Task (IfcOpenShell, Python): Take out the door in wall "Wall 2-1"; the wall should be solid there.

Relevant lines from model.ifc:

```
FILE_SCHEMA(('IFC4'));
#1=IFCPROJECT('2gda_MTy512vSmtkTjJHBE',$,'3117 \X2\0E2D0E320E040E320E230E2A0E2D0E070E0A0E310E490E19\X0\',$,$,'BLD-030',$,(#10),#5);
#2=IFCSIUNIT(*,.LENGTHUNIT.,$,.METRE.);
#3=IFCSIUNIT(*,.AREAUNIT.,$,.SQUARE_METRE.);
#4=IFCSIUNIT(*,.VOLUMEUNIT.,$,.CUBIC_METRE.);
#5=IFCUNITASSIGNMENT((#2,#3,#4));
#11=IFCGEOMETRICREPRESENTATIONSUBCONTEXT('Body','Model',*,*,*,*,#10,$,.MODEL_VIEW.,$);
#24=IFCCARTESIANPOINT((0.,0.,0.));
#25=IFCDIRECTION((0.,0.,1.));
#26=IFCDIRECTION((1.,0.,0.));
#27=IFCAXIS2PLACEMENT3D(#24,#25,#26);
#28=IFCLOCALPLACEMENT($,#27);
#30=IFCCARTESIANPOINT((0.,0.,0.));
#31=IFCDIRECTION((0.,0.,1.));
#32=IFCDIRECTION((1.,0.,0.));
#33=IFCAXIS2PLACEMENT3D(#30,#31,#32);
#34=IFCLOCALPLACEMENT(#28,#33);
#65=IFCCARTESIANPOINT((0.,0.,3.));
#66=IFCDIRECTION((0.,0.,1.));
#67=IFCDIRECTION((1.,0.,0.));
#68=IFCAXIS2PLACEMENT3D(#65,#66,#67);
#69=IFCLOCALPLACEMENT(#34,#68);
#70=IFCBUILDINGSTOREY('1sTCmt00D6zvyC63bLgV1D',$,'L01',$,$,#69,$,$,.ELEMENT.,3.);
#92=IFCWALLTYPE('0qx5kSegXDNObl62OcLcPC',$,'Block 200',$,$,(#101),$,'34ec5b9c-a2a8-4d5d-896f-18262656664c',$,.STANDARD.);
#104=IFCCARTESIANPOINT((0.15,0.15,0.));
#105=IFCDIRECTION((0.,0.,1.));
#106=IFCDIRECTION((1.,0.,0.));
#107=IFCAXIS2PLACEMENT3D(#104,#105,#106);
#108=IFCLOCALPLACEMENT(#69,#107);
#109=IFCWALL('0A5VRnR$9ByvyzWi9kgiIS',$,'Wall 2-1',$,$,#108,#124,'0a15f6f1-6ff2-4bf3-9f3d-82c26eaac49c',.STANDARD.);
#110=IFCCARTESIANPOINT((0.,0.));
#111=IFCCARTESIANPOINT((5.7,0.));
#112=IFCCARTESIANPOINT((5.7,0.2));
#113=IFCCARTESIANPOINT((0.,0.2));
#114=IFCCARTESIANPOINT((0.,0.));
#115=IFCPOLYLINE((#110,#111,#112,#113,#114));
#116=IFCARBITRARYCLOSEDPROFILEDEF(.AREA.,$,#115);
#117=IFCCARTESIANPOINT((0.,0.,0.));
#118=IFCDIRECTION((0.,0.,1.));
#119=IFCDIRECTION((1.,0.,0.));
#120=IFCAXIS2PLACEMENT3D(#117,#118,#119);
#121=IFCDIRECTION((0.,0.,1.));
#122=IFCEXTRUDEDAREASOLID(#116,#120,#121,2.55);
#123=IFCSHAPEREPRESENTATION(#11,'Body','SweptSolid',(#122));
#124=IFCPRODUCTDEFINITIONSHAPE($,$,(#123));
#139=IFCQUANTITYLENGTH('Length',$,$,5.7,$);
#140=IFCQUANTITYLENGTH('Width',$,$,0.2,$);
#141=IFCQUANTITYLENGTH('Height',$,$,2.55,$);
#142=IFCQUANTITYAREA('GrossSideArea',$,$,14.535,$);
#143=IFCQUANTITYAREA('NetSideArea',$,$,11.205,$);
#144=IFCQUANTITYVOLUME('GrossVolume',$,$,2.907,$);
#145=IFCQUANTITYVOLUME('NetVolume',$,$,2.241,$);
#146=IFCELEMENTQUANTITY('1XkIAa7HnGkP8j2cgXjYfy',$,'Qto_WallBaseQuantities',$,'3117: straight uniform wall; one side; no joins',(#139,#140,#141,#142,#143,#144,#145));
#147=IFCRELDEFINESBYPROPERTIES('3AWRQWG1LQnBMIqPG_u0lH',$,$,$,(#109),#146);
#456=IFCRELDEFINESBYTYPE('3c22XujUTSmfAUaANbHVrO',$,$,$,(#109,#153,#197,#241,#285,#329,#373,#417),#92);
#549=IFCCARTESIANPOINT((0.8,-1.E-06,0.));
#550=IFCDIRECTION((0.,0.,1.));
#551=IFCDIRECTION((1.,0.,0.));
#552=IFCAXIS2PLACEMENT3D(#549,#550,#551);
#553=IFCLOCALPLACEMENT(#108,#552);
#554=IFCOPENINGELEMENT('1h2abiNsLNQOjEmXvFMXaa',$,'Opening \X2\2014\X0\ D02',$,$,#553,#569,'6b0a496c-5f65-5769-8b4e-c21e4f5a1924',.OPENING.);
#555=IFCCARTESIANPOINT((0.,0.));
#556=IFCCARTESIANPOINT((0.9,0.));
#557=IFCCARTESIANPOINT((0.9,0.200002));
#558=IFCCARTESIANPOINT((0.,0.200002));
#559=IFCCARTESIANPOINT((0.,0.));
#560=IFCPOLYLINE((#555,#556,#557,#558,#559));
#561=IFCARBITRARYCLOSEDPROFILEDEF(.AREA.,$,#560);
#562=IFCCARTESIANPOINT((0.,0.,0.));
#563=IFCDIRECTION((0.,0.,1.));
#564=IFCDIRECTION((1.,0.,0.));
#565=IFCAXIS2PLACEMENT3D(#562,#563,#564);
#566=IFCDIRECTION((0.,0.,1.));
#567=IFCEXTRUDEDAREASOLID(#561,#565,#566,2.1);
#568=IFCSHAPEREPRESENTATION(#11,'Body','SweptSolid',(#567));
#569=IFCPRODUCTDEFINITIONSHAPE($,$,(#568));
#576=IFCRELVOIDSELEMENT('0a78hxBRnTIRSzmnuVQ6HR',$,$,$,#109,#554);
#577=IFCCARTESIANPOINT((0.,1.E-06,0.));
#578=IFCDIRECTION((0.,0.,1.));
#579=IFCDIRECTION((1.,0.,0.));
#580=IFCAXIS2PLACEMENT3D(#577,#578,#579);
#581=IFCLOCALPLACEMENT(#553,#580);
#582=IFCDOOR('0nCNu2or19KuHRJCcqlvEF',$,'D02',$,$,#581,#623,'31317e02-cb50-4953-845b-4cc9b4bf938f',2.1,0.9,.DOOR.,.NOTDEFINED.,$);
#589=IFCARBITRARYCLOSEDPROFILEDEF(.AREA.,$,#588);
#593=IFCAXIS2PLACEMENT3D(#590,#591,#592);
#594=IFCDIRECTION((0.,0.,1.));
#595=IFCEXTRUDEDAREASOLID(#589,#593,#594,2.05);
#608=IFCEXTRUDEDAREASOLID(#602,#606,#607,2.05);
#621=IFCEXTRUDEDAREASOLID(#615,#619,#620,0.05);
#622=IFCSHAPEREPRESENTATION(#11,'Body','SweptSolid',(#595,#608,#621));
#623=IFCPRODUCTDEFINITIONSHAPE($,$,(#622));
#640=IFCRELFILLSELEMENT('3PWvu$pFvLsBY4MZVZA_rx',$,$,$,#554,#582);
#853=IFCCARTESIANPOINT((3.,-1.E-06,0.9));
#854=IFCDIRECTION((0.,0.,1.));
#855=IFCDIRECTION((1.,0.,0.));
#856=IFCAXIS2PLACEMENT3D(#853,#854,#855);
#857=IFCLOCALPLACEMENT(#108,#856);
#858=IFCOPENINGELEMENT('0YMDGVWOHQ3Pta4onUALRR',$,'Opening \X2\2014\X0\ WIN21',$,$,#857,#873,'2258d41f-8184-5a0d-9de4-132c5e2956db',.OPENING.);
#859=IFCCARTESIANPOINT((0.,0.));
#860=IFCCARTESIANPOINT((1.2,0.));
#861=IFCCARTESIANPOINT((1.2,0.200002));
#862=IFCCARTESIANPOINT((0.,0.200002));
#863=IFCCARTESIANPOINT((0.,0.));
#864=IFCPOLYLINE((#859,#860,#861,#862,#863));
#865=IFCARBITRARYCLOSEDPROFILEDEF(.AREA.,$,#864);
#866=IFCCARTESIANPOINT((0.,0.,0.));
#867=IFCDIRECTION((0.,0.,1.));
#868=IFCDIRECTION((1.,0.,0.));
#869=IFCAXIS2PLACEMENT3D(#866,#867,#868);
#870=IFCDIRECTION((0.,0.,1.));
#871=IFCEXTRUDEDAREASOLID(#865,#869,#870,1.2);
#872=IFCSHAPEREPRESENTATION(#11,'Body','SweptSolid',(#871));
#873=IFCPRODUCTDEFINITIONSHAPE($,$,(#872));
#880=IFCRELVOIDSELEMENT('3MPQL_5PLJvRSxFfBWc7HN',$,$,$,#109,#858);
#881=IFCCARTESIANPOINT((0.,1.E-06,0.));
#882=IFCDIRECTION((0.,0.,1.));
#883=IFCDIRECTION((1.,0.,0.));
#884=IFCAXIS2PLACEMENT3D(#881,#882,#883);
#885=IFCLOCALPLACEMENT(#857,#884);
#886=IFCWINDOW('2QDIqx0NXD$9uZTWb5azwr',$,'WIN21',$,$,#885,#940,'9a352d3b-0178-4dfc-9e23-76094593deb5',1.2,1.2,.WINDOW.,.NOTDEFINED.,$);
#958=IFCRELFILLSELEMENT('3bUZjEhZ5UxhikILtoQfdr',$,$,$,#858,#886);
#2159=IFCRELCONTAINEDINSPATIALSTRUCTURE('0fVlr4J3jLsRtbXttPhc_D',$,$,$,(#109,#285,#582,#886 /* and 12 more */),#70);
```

```python
import ifcopenshell
import ifcopenshell.api.feature
import ifcopenshell.api.pset
import ifcopenshell.api.root
import ifcopenshell.geom
import ifcopenshell.util.element
import ifcopenshell.util.shape
import ifcopenshell.util.unit

model = ifcopenshell.open("model.ifc")
area_scale = ifcopenshell.util.unit.calculate_unit_scale(model, "AREAUNIT")
volume_scale = ifcopenshell.util.unit.calculate_unit_scale(model, "VOLUMEUNIT")
settings = ifcopenshell.geom.settings()


def volume(element):
    """Net volume in cubic metres, openings subtracted."""
    shape = ifcopenshell.geom.create_shape(settings, element)
    return ifcopenshell.util.shape.get_volume(shape.geometry)


door = model.by_id(582)
opening = door.FillsVoids[0].RelatingOpeningElement
wall = opening.VoidsElements[0].RelatingBuildingElement
before = volume(wall)

ifcopenshell.api.root.remove_product(model, product=door)
ifcopenshell.api.feature.remove_feature(model, feature=opening)

after = volume(wall)
thickness = 0.2  # wall thickness in metres

# Update the wall's stored quantities.
qto = model.by_id(ifcopenshell.util.element.get_pset(wall, "Qto_WallBaseQuantities", should_inherit=False)["id"])
ifcopenshell.api.pset.edit_qto(model, qto=qto, properties={
    "NetSideArea": after / thickness / area_scale,
    "NetVolume": after / volume_scale,
})

print(f"wall volume {before:.3f} -> {after:.3f} m3")

model.write("model-out.ifc")
```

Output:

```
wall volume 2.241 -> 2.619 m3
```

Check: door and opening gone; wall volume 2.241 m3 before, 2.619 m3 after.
